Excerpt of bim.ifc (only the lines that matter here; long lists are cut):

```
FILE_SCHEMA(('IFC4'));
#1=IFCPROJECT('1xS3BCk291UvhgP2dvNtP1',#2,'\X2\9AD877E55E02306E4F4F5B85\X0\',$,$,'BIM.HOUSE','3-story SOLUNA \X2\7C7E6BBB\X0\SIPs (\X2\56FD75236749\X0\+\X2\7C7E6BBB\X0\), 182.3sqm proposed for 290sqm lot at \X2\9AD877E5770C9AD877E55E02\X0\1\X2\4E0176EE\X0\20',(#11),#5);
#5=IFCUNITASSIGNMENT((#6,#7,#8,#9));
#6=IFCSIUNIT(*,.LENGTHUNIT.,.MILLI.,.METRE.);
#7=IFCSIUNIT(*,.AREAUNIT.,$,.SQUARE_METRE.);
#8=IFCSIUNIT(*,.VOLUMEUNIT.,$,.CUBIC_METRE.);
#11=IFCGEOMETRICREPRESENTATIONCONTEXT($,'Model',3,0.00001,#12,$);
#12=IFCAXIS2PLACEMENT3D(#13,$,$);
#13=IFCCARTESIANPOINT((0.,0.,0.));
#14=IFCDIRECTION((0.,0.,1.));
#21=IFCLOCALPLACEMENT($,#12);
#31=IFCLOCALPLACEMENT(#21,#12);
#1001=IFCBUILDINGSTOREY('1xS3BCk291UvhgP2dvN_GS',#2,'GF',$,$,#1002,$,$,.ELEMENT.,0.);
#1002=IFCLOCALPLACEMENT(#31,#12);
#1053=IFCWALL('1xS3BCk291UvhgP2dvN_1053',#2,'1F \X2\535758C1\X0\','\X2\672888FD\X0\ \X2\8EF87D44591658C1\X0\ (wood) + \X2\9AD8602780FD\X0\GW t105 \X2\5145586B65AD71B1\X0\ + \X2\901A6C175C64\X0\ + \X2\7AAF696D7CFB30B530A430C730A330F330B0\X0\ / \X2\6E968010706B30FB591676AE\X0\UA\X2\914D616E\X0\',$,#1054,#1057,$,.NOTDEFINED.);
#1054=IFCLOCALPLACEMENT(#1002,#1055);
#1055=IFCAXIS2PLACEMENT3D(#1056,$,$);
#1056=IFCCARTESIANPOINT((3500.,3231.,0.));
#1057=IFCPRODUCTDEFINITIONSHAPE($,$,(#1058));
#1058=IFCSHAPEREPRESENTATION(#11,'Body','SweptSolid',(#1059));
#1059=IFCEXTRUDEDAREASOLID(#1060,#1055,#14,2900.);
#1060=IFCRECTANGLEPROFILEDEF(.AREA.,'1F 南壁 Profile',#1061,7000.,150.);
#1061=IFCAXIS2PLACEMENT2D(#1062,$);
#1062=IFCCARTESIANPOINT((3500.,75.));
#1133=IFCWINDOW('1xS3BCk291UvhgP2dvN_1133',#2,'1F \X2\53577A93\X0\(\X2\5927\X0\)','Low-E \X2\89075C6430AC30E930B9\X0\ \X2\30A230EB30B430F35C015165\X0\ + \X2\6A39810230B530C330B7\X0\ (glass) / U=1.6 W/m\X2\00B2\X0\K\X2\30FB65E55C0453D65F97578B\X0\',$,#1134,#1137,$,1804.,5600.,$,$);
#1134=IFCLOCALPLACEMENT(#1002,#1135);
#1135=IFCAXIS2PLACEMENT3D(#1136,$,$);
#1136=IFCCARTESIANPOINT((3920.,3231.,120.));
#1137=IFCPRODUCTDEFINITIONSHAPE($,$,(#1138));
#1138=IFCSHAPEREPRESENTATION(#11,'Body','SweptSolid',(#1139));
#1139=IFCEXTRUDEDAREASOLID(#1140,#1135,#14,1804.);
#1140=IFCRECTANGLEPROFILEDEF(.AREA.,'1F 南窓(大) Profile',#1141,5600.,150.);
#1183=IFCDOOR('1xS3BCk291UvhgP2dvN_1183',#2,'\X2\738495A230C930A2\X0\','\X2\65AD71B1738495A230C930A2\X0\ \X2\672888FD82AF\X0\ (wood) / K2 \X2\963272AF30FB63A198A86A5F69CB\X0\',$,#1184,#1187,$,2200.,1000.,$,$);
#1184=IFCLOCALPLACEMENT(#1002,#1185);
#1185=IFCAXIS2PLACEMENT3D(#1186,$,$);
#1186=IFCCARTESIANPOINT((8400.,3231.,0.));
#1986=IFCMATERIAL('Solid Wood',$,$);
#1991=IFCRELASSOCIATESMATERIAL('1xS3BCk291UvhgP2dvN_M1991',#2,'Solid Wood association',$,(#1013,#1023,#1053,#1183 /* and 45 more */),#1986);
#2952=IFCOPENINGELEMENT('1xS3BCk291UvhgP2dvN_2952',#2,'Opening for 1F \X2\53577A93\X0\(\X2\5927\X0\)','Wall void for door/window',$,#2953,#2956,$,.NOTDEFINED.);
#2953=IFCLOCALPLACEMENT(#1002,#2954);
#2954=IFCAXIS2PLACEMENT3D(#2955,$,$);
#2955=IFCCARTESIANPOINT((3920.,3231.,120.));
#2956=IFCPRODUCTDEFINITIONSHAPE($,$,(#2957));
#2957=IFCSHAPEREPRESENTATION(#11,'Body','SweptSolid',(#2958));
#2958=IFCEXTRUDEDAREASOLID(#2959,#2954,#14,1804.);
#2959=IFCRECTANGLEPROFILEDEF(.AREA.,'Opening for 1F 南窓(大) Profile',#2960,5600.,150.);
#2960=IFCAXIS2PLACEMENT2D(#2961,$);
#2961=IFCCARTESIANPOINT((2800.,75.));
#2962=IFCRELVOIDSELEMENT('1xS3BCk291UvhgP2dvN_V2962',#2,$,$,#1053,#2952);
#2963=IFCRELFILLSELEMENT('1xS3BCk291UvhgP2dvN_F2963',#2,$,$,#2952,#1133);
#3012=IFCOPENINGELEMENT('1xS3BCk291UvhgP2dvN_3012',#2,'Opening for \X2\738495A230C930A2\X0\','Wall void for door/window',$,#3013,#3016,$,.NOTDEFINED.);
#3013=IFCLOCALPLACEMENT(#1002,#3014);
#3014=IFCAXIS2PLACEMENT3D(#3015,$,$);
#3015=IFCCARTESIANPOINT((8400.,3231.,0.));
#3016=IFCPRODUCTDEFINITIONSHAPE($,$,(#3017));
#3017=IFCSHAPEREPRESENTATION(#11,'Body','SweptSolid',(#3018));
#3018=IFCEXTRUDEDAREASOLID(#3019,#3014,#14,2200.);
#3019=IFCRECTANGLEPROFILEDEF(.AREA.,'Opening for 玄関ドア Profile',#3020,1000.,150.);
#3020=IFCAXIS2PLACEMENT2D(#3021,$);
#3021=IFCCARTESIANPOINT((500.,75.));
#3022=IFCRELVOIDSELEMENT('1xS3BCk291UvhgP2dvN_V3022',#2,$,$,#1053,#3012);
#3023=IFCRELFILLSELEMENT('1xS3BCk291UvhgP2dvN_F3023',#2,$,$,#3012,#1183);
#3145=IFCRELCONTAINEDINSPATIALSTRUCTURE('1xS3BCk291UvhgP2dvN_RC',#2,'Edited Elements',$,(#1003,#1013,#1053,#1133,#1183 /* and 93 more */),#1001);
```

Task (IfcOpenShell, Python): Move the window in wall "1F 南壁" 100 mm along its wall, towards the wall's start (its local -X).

```python
import ifcopenshell
import ifcopenshell.api.geometry
import ifcopenshell.util.placement

model = ifcopenshell.open("bim.ifc")

window = model.by_guid("1xS3BCk291UvhgP2dvN_1133")
opening = window.FillsVoids[0].RelatingOpeningElement
wall = opening.VoidsElements[0].RelatingBuildingElement

wall_matrix = ifcopenshell.util.placement.get_local_placement(wall.ObjectPlacement)
shift = wall_matrix[:3, 0] * -100.0
before = ifcopenshell.util.placement.get_local_placement(window.ObjectPlacement)[:3, 3].copy()

# The window is not placed relative to its opening, so move both.
for product in (opening, window):
    matrix = ifcopenshell.util.placement.get_local_placement(product.ObjectPlacement)
    matrix[:3, 3] += shift
    ifcopenshell.api.geometry.edit_object_placement(model, product=product, matrix=matrix, is_si=False)

after = ifcopenshell.util.placement.get_local_placement(window.ObjectPlacement)[:3, 3]
print("window moved by", (after - before).round(3) + 0.0)

model.write("bim_rev.ifc")
```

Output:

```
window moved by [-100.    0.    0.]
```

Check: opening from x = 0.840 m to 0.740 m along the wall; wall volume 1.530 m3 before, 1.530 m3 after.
